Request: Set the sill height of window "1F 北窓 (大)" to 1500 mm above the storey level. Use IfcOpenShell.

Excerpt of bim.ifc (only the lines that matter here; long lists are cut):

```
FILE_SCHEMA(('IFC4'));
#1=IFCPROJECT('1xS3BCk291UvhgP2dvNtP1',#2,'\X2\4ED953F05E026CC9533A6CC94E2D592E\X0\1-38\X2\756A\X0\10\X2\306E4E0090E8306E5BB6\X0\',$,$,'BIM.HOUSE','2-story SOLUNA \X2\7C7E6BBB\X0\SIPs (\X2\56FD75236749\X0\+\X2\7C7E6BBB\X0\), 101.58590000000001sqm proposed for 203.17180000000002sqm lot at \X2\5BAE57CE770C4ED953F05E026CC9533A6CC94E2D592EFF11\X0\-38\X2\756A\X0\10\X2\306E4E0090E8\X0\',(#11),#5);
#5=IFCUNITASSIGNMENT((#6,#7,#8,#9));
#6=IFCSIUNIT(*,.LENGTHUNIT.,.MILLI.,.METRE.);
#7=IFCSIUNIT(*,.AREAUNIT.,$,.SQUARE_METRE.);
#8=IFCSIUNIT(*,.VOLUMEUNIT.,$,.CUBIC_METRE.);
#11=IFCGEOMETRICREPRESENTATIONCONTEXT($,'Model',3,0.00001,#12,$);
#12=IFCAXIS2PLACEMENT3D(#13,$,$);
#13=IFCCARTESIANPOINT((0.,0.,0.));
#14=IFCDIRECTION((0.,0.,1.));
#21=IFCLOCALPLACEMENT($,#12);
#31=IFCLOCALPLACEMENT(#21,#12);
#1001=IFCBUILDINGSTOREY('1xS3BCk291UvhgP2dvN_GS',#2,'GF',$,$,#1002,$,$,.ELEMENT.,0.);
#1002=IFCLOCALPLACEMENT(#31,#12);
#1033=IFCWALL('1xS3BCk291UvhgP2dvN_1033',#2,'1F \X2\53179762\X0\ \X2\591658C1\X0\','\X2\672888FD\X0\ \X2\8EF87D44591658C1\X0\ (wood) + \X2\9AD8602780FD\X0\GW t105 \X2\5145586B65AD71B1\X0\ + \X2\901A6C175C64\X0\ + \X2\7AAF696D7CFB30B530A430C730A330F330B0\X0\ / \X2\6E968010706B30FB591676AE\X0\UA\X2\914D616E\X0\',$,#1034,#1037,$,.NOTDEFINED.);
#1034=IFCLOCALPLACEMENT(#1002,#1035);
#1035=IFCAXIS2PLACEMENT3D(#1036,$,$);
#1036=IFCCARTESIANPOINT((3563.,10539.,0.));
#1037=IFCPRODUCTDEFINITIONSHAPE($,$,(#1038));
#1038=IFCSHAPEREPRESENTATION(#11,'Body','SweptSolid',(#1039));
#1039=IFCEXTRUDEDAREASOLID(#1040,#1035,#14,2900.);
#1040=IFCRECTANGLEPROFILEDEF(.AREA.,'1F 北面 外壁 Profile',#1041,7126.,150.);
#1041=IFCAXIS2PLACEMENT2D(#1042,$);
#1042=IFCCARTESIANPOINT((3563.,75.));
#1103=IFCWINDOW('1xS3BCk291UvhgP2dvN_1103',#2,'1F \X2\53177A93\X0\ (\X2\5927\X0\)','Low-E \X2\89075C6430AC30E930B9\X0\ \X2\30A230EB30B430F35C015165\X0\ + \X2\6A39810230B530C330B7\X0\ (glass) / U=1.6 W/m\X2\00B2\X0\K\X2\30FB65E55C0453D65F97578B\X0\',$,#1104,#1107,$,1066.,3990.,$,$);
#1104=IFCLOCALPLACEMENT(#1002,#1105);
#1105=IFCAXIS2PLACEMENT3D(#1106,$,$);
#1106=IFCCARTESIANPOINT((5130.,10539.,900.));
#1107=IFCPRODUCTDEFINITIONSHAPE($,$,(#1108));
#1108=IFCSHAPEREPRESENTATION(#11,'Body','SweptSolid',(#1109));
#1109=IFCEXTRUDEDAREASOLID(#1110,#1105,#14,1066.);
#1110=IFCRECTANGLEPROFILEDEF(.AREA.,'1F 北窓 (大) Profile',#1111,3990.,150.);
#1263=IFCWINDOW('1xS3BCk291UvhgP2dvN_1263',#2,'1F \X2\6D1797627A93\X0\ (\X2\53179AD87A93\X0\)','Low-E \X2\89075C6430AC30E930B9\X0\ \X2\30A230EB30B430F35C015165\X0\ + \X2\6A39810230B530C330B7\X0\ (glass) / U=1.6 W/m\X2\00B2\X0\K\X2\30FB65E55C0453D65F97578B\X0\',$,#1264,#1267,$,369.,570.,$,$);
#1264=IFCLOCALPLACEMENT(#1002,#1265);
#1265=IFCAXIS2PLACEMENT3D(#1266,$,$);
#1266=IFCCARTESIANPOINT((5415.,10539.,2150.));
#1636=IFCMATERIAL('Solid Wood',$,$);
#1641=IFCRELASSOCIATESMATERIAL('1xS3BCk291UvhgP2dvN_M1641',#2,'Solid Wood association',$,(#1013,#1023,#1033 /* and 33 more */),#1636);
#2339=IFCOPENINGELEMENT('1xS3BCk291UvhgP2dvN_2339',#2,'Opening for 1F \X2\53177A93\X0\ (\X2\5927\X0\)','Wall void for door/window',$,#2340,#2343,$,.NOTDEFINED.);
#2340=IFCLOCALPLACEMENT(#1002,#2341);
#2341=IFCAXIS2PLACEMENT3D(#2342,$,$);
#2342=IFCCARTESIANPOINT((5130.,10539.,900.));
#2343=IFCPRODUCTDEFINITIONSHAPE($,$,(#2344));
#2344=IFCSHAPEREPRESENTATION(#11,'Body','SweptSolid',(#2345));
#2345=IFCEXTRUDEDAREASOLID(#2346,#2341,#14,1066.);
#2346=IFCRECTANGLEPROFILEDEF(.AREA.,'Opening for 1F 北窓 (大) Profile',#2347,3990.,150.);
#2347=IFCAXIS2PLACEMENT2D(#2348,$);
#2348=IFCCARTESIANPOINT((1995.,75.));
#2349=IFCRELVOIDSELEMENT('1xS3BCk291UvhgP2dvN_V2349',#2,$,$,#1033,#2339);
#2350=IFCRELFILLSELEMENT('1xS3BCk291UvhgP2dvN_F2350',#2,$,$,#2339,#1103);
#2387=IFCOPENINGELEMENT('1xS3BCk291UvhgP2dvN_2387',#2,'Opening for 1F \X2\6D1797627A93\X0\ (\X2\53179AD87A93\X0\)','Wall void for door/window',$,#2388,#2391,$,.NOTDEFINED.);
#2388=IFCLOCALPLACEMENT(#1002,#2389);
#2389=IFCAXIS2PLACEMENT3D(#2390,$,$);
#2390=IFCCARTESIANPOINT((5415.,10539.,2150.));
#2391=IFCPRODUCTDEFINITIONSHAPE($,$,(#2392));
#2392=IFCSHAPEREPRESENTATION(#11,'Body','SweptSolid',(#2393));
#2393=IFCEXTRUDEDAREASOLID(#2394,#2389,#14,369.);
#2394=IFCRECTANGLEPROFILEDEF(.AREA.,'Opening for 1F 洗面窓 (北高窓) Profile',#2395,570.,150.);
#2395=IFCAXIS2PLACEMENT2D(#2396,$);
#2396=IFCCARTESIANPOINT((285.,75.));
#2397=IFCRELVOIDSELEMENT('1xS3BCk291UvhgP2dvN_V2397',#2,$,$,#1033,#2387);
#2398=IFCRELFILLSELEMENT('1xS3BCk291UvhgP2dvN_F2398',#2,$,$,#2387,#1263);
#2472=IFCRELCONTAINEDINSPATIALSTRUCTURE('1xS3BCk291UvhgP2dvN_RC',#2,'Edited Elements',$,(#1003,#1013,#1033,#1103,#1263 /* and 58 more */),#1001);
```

```python
import numpy as np
import ifcopenshell
import ifcopenshell.api.geometry
import ifcopenshell.geom
import ifcopenshell.util.element
import ifcopenshell.util.placement
import ifcopenshell.util.shape
import ifcopenshell.util.unit

model = ifcopenshell.open("bim.ifc")
unit_scale = ifcopenshell.util.unit.calculate_unit_scale(model)

window = model.by_id(1103)
opening = window.FillsVoids[0].RelatingOpeningElement
storey = ifcopenshell.util.element.get_container(window, ifc_class="IfcBuildingStorey")
level = ifcopenshell.util.placement.get_local_placement(storey.ObjectPlacement)[2, 3]

# The opening's origin need not be at the sill, so measure its lowest point.
shape = ifcopenshell.geom.create_shape(ifcopenshell.geom.settings(), opening)
bottom = ifcopenshell.util.shape.get_shape_bottom_elevation(shape, shape.geometry) / unit_scale
dz = level + 1.5 / unit_scale - bottom

shift = np.array([0.0, 0.0, dz])
# The window is not placed relative to its opening, so move both.
for product in (opening, window):
    matrix = ifcopenshell.util.placement.get_local_placement(product.ObjectPlacement)
    matrix[:3, 3] += shift
    ifcopenshell.api.geometry.edit_object_placement(model, product=product, matrix=matrix, is_si=False)

print(f"moved by {dz * unit_scale:+.3f} m")

model.write("bim_edited.ifc")
```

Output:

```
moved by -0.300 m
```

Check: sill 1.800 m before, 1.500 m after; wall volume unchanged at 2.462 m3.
